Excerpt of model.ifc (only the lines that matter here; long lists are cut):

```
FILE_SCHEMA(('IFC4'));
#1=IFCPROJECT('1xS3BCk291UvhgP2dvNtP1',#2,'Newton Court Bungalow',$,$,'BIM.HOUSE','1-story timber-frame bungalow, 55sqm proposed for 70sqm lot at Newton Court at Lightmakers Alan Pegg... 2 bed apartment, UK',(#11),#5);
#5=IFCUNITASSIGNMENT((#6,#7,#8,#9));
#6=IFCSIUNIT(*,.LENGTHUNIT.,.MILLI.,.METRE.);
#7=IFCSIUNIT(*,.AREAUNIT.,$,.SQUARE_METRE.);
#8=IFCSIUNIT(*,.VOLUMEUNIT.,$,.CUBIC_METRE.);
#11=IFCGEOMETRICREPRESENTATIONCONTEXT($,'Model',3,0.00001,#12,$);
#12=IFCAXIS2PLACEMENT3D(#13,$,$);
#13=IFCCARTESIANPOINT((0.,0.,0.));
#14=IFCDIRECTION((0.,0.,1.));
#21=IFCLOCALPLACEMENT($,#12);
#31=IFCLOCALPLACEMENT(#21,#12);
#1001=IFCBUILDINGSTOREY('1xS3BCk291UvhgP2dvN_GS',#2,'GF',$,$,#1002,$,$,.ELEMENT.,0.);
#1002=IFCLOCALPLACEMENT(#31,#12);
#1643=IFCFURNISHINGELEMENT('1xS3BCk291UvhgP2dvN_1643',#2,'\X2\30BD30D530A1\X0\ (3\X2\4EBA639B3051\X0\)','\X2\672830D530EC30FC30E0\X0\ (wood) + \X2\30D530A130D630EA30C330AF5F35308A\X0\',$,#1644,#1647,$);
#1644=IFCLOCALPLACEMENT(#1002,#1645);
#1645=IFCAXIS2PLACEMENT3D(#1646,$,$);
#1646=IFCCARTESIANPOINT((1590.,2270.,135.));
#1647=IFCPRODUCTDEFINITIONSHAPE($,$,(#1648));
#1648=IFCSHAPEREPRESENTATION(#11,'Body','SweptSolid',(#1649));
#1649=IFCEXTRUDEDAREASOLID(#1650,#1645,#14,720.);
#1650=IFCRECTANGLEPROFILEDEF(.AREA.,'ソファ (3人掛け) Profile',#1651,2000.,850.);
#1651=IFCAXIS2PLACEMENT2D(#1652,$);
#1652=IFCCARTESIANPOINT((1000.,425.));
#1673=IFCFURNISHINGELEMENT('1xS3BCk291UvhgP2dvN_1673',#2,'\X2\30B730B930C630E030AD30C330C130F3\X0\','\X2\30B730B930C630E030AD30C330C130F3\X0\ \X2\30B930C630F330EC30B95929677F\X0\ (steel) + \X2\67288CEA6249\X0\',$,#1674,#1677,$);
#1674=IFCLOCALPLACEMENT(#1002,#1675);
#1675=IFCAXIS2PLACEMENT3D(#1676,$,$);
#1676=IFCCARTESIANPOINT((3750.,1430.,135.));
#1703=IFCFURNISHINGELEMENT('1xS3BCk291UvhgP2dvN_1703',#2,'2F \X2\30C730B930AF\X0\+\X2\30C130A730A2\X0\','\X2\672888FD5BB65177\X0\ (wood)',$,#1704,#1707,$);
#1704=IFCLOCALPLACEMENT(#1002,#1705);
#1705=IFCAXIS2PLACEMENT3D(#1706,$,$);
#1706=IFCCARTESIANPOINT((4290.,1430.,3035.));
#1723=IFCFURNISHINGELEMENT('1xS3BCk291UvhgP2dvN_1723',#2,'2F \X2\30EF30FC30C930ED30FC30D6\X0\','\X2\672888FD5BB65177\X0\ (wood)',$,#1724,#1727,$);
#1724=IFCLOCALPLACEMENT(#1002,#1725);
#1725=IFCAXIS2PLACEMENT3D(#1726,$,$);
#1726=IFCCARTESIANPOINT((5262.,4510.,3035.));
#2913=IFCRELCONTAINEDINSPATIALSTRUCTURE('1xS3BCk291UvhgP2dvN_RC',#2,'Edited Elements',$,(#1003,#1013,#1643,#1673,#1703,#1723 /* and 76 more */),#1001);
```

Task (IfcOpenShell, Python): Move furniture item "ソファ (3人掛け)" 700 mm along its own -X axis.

```python
import ifcopenshell
import ifcopenshell.api.geometry
import ifcopenshell.util.placement
import ifcopenshell.util.unit

model = ifcopenshell.open("model.ifc")
unit_scale = ifcopenshell.util.unit.calculate_unit_scale(model)

item = model.by_guid("1xS3BCk291UvhgP2dvN_1643")
matrix = ifcopenshell.util.placement.get_local_placement(item.ObjectPlacement)
matrix[:3, 3] -= matrix[:3, 0] * 0.7 / unit_scale
ifcopenshell.api.geometry.edit_object_placement(model, product=item, matrix=matrix, is_si=False)

print(ifcopenshell.util.placement.get_local_placement(item.ObjectPlacement).round(3) + 0.0)

model.write("model_updated.ifc")
```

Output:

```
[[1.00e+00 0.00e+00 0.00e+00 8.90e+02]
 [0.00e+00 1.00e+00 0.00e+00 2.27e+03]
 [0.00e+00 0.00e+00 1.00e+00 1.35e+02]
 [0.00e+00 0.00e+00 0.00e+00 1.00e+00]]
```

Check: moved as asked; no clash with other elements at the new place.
